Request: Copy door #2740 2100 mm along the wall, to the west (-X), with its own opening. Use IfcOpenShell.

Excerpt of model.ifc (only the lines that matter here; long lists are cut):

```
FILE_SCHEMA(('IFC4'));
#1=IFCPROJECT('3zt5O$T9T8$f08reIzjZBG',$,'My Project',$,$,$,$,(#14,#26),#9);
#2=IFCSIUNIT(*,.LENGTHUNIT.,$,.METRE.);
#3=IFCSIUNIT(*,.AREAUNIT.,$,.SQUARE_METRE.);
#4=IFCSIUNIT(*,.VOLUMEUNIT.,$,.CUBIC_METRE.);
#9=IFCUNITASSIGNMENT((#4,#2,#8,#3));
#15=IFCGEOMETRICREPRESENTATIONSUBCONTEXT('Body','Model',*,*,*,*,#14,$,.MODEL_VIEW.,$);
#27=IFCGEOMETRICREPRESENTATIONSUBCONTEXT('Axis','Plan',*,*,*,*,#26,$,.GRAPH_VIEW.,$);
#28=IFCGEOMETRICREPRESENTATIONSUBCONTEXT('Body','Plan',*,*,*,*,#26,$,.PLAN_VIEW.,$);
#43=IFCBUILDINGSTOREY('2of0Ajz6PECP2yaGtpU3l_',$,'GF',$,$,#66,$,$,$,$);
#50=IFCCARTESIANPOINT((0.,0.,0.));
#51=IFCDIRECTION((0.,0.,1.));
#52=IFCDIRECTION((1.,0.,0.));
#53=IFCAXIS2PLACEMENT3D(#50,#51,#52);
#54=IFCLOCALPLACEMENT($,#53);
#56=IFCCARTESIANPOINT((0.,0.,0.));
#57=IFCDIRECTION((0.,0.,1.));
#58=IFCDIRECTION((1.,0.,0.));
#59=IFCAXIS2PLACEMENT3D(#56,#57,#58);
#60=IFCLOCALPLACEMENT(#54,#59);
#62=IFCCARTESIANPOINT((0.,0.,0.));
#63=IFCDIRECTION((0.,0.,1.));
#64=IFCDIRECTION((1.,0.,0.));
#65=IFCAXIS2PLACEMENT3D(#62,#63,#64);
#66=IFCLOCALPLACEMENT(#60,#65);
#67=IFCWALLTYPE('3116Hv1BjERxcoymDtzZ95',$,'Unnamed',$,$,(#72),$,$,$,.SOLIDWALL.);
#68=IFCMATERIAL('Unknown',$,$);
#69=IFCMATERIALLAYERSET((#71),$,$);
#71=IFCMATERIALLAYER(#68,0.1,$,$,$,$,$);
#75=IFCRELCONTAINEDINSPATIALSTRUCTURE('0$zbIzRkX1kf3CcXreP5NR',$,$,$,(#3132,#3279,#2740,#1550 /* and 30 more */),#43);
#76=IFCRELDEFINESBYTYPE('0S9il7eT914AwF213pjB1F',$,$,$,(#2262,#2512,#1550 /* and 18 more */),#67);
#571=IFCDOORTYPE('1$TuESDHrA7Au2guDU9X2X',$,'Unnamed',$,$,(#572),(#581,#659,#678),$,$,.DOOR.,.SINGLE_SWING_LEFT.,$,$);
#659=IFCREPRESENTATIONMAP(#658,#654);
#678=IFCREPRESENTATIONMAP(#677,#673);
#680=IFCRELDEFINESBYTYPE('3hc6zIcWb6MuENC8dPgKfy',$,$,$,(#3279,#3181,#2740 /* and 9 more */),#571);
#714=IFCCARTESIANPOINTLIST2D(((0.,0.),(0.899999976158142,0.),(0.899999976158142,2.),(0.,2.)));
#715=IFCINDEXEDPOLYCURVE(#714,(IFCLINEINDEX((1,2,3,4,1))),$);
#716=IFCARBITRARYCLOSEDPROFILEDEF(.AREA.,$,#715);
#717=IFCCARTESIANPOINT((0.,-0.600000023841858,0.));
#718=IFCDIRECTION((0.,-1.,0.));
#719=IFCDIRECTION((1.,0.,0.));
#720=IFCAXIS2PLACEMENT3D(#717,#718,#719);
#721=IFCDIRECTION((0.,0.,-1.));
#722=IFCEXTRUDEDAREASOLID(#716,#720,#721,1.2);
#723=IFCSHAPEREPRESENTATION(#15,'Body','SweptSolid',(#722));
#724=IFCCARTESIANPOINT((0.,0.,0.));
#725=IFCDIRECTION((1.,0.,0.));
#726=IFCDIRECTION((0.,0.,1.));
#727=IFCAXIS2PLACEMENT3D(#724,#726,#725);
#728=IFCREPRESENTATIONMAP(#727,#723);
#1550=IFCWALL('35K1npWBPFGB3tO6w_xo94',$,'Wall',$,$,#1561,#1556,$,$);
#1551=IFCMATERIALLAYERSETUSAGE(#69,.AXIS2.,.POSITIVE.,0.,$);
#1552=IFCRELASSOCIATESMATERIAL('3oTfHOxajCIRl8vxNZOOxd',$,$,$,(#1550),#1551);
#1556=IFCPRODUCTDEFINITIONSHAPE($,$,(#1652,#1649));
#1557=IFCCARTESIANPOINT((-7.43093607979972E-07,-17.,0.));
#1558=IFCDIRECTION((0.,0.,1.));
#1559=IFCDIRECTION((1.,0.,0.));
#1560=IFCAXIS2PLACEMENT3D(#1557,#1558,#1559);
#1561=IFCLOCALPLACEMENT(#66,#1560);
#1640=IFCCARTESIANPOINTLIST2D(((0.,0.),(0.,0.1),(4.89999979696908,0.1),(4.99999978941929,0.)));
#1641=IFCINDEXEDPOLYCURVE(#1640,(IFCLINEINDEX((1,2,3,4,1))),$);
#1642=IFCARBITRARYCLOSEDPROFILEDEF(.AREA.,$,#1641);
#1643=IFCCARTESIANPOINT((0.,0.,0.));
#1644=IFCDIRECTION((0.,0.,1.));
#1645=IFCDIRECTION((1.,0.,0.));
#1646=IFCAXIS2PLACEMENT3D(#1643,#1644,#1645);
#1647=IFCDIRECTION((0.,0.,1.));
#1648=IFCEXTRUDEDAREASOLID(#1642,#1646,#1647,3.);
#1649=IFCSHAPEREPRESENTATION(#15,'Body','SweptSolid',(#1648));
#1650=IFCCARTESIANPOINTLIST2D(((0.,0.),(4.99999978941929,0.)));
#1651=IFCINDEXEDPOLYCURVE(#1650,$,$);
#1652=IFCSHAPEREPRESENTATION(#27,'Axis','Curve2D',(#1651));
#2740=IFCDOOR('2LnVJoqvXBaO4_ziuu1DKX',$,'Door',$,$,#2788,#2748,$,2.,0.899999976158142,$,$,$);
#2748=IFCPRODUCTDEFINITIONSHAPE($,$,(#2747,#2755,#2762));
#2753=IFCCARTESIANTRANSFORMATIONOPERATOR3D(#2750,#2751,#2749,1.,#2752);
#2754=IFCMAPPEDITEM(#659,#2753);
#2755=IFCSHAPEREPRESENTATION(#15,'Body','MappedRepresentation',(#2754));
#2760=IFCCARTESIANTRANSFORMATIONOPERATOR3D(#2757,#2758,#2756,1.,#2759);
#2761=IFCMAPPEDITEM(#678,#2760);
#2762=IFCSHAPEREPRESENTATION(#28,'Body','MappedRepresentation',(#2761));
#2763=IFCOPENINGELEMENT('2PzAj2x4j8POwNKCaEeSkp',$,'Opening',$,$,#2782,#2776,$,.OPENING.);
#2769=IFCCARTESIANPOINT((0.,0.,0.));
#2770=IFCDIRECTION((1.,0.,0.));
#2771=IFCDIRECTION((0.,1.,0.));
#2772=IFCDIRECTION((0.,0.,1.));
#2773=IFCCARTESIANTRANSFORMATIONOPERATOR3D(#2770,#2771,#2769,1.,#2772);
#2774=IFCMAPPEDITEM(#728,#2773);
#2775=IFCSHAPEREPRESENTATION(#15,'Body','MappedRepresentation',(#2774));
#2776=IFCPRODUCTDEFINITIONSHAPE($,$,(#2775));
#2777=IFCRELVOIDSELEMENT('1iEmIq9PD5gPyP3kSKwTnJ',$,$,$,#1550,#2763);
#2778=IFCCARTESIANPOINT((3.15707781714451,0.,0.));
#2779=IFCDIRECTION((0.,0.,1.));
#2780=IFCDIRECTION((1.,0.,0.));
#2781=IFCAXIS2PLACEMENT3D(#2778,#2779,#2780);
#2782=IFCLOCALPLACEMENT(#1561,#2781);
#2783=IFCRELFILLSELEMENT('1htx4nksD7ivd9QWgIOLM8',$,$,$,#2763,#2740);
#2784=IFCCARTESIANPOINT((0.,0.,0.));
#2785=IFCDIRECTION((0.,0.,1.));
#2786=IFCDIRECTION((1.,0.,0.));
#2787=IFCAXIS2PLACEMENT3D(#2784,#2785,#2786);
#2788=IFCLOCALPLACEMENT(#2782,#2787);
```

```python
import ifcopenshell
import ifcopenshell.api.feature
import ifcopenshell.api.geometry
import ifcopenshell.api.root
import ifcopenshell.geom
import ifcopenshell.util.element
import ifcopenshell.util.placement
import ifcopenshell.util.shape
import ifcopenshell.util.unit

model = ifcopenshell.open("model.ifc")
unit_scale = ifcopenshell.util.unit.calculate_unit_scale(model)
settings = ifcopenshell.geom.settings()


def volume(element):
    """Net volume in cubic metres, openings subtracted."""
    shape = ifcopenshell.geom.create_shape(settings, element)
    return ifcopenshell.util.shape.get_volume(shape.geometry)


door = model.by_guid("2LnVJoqvXBaO4_ziuu1DKX")
opening = door.FillsVoids[0].RelatingOpeningElement
wall = opening.VoidsElements[0].RelatingBuildingElement
before = volume(wall)
shift = ifcopenshell.util.placement.get_local_placement(wall.ObjectPlacement)[:3, 0] * -2.1 / unit_scale

# copy_class copies the void relationship, type, container and properties, but no geometry.
new_opening = ifcopenshell.api.root.copy_class(model, product=opening)
new_opening.Representation = ifcopenshell.util.element.copy_deep(
    model, opening.Representation, exclude=["IfcGeometricRepresentationContext", "IfcRepresentationMap"]
)
new_door = ifcopenshell.api.root.copy_class(model, product=door)
new_door.Representation = ifcopenshell.util.element.copy_deep(
    model, door.Representation, exclude=["IfcGeometricRepresentationContext", "IfcRepresentationMap"]
)
ifcopenshell.api.feature.add_filling(model, opening=new_opening, element=new_door)

for old, new in ((opening, new_opening), (door, new_door)):
    matrix = ifcopenshell.util.placement.get_local_placement(old.ObjectPlacement)
    matrix[:3, 3] += shift
    ifcopenshell.api.geometry.edit_object_placement(model, product=new, matrix=matrix, is_si=False)

after = volume(wall)

print(f"wall volume {before:.3f} -> {after:.3f} m3")

model.write("model_edited.ifc")
```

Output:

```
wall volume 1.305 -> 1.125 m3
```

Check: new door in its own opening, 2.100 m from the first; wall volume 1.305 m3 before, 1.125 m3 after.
